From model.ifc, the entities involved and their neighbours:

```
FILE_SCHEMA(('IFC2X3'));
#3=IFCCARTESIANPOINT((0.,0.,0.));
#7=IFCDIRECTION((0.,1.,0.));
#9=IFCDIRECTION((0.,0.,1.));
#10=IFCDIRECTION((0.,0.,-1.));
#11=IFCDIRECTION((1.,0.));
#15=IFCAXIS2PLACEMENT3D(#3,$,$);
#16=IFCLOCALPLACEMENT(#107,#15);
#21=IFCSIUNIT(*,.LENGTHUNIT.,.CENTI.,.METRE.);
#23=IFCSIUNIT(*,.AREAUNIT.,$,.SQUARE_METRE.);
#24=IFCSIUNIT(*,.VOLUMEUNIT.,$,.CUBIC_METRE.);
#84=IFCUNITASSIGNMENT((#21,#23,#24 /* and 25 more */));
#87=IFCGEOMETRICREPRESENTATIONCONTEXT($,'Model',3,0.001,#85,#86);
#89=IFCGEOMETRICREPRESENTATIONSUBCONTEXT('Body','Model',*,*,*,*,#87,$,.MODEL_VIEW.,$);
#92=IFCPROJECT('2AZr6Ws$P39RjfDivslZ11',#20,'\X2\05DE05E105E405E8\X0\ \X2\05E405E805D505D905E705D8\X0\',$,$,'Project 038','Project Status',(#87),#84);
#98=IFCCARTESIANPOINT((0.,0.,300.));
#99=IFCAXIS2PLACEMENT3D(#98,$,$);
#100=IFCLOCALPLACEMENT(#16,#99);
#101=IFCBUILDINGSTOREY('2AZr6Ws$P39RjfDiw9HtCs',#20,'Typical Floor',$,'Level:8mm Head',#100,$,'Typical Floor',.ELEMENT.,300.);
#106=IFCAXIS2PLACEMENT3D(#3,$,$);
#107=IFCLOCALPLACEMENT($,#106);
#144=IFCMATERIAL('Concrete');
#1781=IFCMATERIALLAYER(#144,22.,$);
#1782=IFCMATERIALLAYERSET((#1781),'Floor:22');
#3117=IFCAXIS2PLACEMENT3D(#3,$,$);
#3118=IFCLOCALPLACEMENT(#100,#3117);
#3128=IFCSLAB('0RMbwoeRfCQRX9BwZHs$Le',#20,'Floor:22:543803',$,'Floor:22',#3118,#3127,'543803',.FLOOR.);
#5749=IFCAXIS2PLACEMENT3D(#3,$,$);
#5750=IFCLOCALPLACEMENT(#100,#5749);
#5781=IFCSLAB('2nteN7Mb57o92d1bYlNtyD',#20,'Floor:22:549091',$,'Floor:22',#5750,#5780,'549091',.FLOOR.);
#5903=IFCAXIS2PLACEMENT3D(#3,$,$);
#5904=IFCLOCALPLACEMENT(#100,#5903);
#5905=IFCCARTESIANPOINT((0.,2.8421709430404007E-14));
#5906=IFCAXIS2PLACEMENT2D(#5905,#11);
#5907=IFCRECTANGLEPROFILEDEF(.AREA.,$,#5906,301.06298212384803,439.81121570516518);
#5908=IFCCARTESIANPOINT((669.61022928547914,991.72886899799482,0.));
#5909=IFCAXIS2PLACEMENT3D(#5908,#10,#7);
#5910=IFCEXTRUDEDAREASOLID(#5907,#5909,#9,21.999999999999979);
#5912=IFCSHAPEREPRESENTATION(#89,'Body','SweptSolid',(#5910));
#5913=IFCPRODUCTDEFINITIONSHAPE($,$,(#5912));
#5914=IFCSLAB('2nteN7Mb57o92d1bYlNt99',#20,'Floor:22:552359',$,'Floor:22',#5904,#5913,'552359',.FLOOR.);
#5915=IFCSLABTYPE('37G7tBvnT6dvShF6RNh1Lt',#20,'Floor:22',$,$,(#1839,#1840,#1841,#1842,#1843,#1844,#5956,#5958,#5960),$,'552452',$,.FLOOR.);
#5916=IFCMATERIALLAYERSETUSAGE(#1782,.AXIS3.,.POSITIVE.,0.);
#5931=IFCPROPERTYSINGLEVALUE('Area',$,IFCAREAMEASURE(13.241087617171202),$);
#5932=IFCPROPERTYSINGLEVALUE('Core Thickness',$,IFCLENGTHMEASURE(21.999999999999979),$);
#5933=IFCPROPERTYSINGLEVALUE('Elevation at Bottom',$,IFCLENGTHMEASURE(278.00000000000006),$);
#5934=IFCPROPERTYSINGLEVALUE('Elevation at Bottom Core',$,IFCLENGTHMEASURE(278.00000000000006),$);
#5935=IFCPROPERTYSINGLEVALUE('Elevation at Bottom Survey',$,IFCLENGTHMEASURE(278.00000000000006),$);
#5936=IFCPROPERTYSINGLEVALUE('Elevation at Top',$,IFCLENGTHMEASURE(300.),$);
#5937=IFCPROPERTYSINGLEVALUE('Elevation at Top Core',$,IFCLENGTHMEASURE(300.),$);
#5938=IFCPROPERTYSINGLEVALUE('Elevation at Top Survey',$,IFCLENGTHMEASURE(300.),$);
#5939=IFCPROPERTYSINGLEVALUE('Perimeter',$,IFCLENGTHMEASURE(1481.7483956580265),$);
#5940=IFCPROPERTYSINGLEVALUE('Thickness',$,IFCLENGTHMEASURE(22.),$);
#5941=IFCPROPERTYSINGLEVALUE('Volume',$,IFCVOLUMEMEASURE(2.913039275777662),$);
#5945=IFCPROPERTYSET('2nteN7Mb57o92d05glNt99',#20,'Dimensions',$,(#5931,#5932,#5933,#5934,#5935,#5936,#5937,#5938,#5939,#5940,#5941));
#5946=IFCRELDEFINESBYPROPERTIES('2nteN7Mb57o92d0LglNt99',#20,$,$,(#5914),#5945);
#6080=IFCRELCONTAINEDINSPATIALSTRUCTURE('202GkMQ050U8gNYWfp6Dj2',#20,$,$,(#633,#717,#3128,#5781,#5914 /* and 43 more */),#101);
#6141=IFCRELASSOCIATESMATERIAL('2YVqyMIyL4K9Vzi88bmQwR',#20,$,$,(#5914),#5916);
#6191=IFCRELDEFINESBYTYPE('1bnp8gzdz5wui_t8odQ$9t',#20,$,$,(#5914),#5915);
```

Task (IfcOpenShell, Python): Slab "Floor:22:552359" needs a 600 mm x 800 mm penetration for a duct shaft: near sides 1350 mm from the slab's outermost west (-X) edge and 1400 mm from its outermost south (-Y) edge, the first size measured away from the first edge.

```python
import numpy as np
import ifcopenshell
import ifcopenshell.api.feature
import ifcopenshell.api.geometry
import ifcopenshell.api.pset
import ifcopenshell.api.root
import ifcopenshell.geom
import ifcopenshell.util.element
import ifcopenshell.util.placement
import ifcopenshell.util.representation
import ifcopenshell.util.shape
import ifcopenshell.util.unit

model = ifcopenshell.open("model.ifc")
unit_scale = ifcopenshell.util.unit.calculate_unit_scale(model)
area_scale = ifcopenshell.util.unit.calculate_unit_scale(model, "AREAUNIT")
volume_scale = ifcopenshell.util.unit.calculate_unit_scale(model, "VOLUMEUNIT")
settings = ifcopenshell.geom.settings()


def volume(element):
    """Net volume in cubic metres, openings subtracted."""
    shape = ifcopenshell.geom.create_shape(settings, element)
    return ifcopenshell.util.shape.get_volume(shape.geometry)


slab = model.by_guid("2nteN7Mb57o92d1bYlNt99")
before = volume(slab)

# Extent in the slab's own axes, in metres. The edges named are its -X and -Y sides.
slab_shape = ifcopenshell.geom.create_shape(settings, slab)
vertices = ifcopenshell.util.shape.get_vertices(slab_shape.geometry)
x_min, y_min, bottom = vertices.min(axis=0)
top = vertices[:, 2].max()

opening = ifcopenshell.api.root.create_entity(model, ifc_class="IfcOpeningElement", name="Duct shaft opening")
context = ifcopenshell.util.representation.get_context(model, "Model", "Body", "MODEL_VIEW")
width, depth = 0.6, 0.8
outline = [(0.0, 0.0), (width, 0.0), (width, depth), (0.0, depth), (0.0, 0.0)]
# Overshoot both faces by 50 mm so the cut is clean.
shape = ifcopenshell.api.geometry.add_slab_representation(
    model, context=context, depth=top - bottom + 0.1, polyline=outline
)
ifcopenshell.api.geometry.assign_representation(model, product=opening, representation=shape)

matrix = ifcopenshell.util.placement.get_local_placement(slab.ObjectPlacement)
matrix[:, 3] = matrix @ np.append(np.array([x_min + 1.35, y_min + 1.4, bottom - 0.05]) / unit_scale, 1.0)
ifcopenshell.api.geometry.edit_object_placement(model, product=opening, matrix=matrix, is_si=False)
ifcopenshell.api.feature.add_feature(model, feature=opening, element=slab)

after = volume(slab)

# Update the slab's stored quantities.
pset = model.by_id(ifcopenshell.util.element.get_pset(slab, "Dimensions", should_inherit=False)["id"])
ifcopenshell.api.pset.edit_pset(model, pset=pset, properties={
    "Area": model.create_entity("IfcAreaMeasure", after / (top - bottom) / area_scale),
    "Volume": model.create_entity("IfcVolumeMeasure", after / volume_scale),
})

print(f"slab volume {before:.3f} -> {after:.3f} m3")

model.write("model-out.ifc")
```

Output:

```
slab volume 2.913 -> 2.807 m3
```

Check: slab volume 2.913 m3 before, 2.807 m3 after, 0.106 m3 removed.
